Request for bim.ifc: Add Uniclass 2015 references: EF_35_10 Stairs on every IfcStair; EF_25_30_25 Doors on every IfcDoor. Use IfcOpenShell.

First a look at what the model holds.

```python
import ifcopenshell

model = ifcopenshell.open("bim.ifc")
print(model.schema)
print("classifications:", [c.Name for c in model.by_type("IfcClassification")])
for ifc_class in ("IfcDoor", "IfcRoof", "IfcStair", "IfcWall", "IfcWindow"):
    print(ifc_class, len(model.by_type(ifc_class)))
```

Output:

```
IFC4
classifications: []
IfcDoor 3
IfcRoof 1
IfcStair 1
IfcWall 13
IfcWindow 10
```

```python
import ifcopenshell
import ifcopenshell.api.classification

model = ifcopenshell.open("bim.ifc")

system = ifcopenshell.api.classification.add_classification(model, classification="Uniclass 2015")

codes = {
    "IfcStair": ("EF_35_10", "Stairs"),
    "IfcDoor": ("EF_25_30_25", "Doors"),
}
for ifc_class, (code, name) in codes.items():
    products = model.by_type(ifc_class)
    ifcopenshell.api.classification.add_reference(
        model, products=products, classification=system, identification=code, name=name
    )
    print(code, len(products))

model.write("bim_v2.ifc")
```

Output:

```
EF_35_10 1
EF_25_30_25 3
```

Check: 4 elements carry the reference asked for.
